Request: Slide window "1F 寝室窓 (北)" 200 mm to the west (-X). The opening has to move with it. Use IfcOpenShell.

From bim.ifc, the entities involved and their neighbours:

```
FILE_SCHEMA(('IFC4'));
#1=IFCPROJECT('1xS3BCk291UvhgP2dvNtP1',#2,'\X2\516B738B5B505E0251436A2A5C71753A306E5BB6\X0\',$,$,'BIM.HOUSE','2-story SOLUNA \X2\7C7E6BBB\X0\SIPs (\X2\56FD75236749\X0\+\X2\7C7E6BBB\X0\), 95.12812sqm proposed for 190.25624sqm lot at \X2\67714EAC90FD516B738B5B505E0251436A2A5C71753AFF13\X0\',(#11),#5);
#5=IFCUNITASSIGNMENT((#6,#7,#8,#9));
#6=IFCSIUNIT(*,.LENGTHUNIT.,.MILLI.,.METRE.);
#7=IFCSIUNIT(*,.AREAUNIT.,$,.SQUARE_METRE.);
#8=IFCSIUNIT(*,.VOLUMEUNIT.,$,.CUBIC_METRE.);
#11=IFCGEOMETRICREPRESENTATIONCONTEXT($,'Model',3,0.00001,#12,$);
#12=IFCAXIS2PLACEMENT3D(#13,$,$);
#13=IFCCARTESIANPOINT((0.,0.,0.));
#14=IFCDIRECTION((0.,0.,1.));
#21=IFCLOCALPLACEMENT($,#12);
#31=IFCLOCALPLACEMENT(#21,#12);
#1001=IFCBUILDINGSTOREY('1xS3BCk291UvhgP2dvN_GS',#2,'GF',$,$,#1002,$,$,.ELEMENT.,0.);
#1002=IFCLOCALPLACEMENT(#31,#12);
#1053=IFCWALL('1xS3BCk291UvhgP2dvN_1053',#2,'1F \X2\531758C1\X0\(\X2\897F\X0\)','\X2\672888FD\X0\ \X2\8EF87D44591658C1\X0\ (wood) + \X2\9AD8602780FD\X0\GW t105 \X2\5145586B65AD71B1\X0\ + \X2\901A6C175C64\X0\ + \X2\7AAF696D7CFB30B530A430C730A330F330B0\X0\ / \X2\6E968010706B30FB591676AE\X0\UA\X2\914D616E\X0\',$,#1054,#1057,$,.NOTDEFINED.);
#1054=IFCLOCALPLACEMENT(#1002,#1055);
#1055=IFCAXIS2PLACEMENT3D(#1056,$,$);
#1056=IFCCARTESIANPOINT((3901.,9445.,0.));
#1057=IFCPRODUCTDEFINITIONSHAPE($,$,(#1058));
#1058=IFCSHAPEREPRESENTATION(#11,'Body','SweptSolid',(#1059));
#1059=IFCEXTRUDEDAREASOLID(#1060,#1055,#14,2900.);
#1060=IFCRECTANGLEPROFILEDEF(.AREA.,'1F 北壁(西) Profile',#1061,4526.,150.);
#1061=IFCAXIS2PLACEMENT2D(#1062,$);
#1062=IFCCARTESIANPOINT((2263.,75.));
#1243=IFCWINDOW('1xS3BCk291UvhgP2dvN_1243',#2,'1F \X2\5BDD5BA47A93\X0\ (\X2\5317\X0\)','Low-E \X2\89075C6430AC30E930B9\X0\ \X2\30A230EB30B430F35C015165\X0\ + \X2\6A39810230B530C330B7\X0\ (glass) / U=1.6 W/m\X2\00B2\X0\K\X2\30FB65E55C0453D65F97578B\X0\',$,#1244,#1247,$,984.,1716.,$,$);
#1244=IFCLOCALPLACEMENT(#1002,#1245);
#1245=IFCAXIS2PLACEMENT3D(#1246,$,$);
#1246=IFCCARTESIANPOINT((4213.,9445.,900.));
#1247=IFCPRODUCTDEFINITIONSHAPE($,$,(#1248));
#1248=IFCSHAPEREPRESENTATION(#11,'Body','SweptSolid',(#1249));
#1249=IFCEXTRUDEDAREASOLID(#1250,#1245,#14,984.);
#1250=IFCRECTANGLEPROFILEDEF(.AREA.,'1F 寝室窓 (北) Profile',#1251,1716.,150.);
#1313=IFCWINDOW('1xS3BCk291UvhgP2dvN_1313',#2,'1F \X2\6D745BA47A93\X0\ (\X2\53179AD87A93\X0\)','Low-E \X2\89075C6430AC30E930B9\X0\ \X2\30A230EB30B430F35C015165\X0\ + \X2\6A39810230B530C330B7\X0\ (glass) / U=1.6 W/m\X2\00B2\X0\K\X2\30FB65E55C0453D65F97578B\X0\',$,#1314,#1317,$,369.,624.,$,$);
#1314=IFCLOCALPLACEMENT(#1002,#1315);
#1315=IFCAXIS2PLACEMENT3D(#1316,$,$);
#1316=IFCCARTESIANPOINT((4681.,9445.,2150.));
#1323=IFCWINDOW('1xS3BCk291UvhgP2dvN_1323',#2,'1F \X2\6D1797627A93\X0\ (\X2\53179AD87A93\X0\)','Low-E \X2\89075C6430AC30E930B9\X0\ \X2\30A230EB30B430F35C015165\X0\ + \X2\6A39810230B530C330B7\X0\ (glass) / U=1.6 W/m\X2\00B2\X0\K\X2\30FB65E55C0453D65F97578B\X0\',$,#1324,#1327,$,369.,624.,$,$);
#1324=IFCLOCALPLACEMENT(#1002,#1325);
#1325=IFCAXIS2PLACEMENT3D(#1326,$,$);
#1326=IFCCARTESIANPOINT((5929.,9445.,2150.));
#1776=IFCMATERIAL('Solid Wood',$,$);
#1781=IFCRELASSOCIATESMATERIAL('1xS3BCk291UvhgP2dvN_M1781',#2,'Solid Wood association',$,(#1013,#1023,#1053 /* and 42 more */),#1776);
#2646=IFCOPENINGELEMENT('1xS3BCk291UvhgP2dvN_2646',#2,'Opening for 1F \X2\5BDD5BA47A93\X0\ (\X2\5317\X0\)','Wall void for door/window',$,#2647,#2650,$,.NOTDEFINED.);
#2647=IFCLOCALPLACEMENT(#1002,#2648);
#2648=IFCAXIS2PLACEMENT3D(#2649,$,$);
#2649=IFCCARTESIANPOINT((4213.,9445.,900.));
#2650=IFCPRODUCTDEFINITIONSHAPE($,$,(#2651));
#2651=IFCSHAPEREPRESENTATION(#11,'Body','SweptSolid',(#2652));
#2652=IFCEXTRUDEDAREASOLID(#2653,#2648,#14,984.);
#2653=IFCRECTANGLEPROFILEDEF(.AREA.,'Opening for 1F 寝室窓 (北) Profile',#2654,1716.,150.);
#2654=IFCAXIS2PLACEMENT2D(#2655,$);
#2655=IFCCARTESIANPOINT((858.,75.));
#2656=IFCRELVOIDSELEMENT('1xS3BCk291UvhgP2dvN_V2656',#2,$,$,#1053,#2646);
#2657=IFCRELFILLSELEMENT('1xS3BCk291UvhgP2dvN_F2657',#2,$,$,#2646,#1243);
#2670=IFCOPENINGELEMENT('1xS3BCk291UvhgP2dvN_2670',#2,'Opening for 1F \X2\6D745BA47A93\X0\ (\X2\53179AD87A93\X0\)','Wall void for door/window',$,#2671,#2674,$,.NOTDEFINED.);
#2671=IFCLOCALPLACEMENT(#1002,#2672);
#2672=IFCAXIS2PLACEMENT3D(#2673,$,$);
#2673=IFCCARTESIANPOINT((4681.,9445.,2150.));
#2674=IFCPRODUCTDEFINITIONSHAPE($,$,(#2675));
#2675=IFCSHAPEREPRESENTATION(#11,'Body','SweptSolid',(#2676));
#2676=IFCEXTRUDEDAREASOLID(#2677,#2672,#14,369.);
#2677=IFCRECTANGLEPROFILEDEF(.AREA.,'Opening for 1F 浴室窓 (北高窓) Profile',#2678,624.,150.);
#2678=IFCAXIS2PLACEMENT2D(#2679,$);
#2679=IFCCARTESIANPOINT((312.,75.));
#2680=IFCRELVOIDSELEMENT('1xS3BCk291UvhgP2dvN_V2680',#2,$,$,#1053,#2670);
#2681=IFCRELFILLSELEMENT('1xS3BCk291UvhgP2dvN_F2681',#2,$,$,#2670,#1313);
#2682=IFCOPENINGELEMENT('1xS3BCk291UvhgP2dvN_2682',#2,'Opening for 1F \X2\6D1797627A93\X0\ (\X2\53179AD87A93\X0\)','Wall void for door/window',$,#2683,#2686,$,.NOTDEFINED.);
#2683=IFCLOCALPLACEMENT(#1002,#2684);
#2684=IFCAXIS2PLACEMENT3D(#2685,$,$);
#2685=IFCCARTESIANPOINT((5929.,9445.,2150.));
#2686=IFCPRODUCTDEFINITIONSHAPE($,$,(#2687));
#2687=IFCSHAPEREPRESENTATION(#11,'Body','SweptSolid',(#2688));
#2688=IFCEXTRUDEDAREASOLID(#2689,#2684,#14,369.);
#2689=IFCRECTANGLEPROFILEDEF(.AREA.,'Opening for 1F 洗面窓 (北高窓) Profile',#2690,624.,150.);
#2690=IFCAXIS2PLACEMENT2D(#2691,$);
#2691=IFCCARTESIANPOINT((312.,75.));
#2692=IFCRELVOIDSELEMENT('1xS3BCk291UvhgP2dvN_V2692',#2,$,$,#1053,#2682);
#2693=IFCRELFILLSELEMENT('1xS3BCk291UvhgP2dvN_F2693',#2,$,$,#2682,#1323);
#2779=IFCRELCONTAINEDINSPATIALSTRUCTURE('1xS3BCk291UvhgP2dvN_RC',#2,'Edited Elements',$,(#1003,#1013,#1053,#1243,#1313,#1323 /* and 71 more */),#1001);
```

```python
import ifcopenshell
import ifcopenshell.api.geometry
import ifcopenshell.util.placement
import ifcopenshell.util.unit

model = ifcopenshell.open("bim.ifc")
unit_scale = ifcopenshell.util.unit.calculate_unit_scale(model)

window = model.by_id(1243)
opening = window.FillsVoids[0].RelatingOpeningElement
wall = opening.VoidsElements[0].RelatingBuildingElement

wall_matrix = ifcopenshell.util.placement.get_local_placement(wall.ObjectPlacement)
shift = wall_matrix[:3, 0] * -0.2 / unit_scale
before = ifcopenshell.util.placement.get_local_placement(window.ObjectPlacement)[:3, 3].copy()

# The window is not placed relative to its opening, so move both.
for product in (opening, window):
    matrix = ifcopenshell.util.placement.get_local_placement(product.ObjectPlacement)
    matrix[:3, 3] += shift
    ifcopenshell.api.geometry.edit_object_placement(model, product=product, matrix=matrix, is_si=False)

after = ifcopenshell.util.placement.get_local_placement(window.ObjectPlacement)[:3, 3]
print("window moved by", (after - before).round(3) + 0.0)

model.write("bim_edited.ifc")
```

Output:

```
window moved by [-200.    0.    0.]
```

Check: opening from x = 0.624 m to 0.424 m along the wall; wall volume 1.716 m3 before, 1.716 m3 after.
